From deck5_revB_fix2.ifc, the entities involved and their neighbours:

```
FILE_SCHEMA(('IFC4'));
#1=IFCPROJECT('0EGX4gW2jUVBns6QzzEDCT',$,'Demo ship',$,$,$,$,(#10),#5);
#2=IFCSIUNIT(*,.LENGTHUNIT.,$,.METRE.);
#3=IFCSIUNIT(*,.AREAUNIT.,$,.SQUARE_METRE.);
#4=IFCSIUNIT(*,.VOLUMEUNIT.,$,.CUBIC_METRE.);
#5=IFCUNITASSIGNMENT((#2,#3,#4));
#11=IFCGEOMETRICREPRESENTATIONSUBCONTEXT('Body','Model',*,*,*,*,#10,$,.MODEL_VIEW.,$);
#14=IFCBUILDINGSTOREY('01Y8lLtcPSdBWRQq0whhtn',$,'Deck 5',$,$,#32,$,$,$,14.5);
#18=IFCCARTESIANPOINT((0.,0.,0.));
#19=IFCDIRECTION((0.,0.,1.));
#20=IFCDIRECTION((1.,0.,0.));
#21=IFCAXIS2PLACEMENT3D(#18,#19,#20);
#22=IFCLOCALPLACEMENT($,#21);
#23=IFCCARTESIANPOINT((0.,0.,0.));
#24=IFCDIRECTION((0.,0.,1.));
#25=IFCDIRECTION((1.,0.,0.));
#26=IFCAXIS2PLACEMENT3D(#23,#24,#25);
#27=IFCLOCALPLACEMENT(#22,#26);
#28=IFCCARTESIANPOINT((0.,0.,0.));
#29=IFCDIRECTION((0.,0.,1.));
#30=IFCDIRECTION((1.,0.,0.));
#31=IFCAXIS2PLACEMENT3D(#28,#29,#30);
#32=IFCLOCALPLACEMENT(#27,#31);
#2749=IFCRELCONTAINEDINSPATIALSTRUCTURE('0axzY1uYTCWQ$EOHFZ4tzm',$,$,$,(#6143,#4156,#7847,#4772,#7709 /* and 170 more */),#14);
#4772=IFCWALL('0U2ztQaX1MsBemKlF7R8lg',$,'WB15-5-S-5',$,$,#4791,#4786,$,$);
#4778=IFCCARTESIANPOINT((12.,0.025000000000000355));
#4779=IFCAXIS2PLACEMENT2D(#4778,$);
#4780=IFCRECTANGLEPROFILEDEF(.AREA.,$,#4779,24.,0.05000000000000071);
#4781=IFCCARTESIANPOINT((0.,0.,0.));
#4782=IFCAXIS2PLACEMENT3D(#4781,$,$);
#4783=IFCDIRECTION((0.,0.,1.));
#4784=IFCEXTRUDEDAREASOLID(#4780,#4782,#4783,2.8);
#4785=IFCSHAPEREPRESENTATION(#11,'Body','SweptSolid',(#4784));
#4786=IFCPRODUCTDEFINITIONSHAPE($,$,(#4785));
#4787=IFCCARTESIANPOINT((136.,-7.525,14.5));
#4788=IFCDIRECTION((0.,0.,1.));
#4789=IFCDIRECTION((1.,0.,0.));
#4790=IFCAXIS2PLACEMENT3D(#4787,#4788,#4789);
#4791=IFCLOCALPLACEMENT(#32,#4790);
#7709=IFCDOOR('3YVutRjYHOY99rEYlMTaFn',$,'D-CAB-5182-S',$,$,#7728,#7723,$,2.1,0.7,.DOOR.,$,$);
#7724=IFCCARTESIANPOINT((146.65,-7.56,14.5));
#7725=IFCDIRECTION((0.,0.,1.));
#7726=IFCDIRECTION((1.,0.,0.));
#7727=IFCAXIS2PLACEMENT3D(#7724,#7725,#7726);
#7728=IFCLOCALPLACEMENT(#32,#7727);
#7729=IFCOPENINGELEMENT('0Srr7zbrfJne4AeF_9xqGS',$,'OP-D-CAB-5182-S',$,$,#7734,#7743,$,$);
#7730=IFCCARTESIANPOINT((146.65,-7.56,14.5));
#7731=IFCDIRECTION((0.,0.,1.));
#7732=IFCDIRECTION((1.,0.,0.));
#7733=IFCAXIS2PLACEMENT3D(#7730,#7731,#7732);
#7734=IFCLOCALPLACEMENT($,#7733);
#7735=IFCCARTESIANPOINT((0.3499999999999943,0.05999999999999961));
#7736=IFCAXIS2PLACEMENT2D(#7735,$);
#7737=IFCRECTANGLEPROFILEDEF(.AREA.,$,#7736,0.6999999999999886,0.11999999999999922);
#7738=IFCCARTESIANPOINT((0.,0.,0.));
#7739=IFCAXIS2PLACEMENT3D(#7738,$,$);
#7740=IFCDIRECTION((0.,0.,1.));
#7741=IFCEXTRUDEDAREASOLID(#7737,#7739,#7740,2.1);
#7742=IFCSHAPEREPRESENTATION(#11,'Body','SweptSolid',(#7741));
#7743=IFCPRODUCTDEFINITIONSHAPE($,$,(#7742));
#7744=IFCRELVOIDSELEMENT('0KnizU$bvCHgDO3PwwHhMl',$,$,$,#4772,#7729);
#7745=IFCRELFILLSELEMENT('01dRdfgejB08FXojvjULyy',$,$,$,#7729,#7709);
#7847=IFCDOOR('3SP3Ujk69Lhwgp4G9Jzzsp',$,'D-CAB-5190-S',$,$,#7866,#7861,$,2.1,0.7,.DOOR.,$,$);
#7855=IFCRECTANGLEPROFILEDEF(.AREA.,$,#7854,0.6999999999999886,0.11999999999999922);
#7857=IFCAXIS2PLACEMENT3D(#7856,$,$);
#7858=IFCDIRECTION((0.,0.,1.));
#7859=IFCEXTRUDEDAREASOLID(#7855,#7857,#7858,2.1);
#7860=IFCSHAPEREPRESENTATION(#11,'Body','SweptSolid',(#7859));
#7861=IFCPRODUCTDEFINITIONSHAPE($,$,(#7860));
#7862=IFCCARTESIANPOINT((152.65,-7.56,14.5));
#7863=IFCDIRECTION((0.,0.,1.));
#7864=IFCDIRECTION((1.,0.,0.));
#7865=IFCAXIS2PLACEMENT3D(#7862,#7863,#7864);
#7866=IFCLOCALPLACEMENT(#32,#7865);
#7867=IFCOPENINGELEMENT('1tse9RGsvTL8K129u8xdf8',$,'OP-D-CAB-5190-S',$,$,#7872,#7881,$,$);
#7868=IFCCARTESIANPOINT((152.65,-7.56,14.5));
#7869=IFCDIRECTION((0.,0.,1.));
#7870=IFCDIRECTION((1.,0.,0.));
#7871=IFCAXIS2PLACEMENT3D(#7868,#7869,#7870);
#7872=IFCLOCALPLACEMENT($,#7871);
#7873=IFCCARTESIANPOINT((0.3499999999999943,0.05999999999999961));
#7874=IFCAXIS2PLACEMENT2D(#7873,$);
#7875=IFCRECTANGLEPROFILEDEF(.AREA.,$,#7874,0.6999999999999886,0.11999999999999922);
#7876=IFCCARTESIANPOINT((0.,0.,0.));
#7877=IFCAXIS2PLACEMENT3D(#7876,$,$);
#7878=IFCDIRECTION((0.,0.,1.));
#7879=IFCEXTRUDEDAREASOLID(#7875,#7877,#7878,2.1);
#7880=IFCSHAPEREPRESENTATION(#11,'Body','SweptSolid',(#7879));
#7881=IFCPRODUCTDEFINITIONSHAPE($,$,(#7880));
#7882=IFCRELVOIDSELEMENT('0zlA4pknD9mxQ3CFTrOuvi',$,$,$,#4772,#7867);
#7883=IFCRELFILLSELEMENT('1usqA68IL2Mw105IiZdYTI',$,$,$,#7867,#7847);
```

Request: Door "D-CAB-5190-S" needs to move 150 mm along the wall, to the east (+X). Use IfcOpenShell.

```python
import ifcopenshell
import ifcopenshell.api.geometry
import ifcopenshell.util.placement
import ifcopenshell.util.unit

model = ifcopenshell.open("deck5_revB_fix2.ifc")
unit_scale = ifcopenshell.util.unit.calculate_unit_scale(model)

door = model.by_guid("3SP3Ujk69Lhwgp4G9Jzzsp")
opening = door.FillsVoids[0].RelatingOpeningElement
wall = opening.VoidsElements[0].RelatingBuildingElement

wall_matrix = ifcopenshell.util.placement.get_local_placement(wall.ObjectPlacement)
shift = wall_matrix[:3, 0] * 0.15 / unit_scale
before = ifcopenshell.util.placement.get_local_placement(door.ObjectPlacement)[:3, 3].copy()

# The door is not placed relative to its opening, so move both.
for product in (opening, door):
    matrix = ifcopenshell.util.placement.get_local_placement(product.ObjectPlacement)
    matrix[:3, 3] += shift
    ifcopenshell.api.geometry.edit_object_placement(model, product=product, matrix=matrix, is_si=False)

after = ifcopenshell.util.placement.get_local_placement(door.ObjectPlacement)[:3, 3]
print("door moved by", (after - before).round(3) + 0.0)

model.write("deck5_revB_fix2_updated.ifc")
```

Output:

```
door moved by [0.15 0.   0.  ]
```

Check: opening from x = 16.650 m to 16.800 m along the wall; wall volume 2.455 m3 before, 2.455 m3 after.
